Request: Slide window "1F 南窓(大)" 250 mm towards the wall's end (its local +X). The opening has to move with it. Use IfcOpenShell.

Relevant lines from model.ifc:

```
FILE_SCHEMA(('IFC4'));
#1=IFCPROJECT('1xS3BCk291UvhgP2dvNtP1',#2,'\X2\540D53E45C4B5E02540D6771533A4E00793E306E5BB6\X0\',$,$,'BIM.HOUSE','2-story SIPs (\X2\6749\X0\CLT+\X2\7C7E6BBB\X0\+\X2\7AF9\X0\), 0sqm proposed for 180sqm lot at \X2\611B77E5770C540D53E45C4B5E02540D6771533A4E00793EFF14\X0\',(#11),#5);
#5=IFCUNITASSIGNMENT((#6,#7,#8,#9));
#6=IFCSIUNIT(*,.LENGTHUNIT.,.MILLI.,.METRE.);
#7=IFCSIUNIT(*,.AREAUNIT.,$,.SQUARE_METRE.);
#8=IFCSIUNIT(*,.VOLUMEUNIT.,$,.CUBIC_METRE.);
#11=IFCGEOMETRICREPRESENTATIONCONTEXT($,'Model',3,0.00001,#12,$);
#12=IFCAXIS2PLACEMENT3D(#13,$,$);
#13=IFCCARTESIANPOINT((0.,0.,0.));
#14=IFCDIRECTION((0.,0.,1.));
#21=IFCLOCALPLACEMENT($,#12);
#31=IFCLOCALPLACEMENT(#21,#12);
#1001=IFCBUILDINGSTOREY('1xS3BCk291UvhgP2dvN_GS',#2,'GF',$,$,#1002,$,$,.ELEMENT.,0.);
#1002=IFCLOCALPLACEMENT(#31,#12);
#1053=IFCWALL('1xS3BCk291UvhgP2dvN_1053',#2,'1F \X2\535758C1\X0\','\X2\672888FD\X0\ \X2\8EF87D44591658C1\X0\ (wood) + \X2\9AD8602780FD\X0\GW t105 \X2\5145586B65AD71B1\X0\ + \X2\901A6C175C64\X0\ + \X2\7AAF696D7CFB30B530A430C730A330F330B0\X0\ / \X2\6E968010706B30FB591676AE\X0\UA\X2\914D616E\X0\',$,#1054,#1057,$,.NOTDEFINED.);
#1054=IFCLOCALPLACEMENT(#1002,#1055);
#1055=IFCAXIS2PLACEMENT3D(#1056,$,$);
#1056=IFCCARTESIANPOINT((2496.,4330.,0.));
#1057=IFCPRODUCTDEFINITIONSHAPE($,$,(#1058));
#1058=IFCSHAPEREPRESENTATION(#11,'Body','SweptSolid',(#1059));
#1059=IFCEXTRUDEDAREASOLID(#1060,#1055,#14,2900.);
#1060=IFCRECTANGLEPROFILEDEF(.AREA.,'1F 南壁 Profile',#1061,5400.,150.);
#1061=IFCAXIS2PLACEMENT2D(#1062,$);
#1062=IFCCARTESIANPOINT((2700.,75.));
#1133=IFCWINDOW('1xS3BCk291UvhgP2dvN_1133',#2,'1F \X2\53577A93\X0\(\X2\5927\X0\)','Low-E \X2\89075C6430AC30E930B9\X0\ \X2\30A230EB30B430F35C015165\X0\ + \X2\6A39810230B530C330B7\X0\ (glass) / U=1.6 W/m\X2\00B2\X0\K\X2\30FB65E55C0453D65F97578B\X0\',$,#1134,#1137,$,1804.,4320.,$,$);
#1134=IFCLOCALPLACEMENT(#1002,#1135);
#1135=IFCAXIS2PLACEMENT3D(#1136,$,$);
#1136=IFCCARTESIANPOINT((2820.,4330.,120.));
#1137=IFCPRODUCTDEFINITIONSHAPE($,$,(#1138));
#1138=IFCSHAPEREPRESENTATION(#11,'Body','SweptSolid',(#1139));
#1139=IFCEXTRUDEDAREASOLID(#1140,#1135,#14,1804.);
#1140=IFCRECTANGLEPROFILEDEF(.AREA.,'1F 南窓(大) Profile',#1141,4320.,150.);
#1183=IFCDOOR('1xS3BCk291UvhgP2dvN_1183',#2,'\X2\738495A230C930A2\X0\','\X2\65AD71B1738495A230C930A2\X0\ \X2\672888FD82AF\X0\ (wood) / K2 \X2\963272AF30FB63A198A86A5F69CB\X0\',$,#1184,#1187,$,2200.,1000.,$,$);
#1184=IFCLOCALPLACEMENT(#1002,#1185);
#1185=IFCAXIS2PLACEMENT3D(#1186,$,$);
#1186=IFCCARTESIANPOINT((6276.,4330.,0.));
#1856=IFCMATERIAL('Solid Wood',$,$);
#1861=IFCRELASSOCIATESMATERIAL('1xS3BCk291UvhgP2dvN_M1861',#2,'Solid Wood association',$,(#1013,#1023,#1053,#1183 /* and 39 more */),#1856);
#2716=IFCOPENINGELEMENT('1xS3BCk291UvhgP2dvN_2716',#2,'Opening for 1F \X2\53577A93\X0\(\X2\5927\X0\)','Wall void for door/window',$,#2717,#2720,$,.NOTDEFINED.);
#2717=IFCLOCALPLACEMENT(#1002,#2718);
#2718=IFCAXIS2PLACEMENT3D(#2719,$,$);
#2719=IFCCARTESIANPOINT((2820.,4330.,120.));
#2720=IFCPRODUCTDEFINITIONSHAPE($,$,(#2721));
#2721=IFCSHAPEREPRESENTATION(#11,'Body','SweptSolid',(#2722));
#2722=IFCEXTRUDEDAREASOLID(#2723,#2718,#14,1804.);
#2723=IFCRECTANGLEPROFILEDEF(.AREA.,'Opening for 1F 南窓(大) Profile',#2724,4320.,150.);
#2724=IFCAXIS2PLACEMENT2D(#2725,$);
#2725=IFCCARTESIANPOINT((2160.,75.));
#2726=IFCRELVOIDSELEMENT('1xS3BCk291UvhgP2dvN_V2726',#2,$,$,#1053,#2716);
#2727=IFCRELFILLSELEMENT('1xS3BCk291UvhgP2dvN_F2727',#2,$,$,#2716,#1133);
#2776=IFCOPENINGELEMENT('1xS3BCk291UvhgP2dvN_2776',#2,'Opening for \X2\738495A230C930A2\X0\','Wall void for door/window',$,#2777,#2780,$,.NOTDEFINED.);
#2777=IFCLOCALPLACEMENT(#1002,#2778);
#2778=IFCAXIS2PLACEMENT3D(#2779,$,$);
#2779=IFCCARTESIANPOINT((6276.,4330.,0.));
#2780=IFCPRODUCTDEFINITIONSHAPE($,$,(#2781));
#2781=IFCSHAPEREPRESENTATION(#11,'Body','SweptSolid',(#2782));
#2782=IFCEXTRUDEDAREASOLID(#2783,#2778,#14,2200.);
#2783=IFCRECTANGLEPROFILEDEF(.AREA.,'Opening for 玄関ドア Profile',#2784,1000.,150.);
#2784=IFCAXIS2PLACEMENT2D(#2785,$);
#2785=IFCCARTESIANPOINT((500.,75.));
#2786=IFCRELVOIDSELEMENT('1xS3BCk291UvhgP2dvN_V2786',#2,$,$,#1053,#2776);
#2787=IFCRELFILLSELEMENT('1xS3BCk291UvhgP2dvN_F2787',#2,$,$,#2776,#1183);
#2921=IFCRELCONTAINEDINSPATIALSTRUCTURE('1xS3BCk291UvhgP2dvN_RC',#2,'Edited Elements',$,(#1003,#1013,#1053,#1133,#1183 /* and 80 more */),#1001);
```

```python
import ifcopenshell
import ifcopenshell.api.geometry
import ifcopenshell.util.placement
import ifcopenshell.util.unit

model = ifcopenshell.open("model.ifc")
unit_scale = ifcopenshell.util.unit.calculate_unit_scale(model)

window = model.by_id(1133)
opening = window.FillsVoids[0].RelatingOpeningElement
wall = opening.VoidsElements[0].RelatingBuildingElement

wall_matrix = ifcopenshell.util.placement.get_local_placement(wall.ObjectPlacement)
shift = wall_matrix[:3, 0] * 0.25 / unit_scale
before = ifcopenshell.util.placement.get_local_placement(window.ObjectPlacement)[:3, 3].copy()

# The window is not placed relative to its opening, so move both.
for product in (opening, window):
    matrix = ifcopenshell.util.placement.get_local_placement(product.ObjectPlacement)
    matrix[:3, 3] += shift
    ifcopenshell.api.geometry.edit_object_placement(model, product=product, matrix=matrix, is_si=False)

after = ifcopenshell.util.placement.get_local_placement(window.ObjectPlacement)[:3, 3]
print("window moved by", (after - before).round(3) + 0.0)

model.write("model_updated.ifc")
```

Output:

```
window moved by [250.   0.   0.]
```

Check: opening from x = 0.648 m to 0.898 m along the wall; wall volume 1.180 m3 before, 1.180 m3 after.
